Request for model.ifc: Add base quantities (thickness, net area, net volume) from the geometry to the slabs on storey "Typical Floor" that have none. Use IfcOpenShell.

First a look at what the model holds.

```python
import ifcopenshell
import ifcopenshell.util.element
import ifcopenshell.util.unit

model = ifcopenshell.open("model.ifc")
print(model.schema)
for unit_type in ("LENGTHUNIT", "AREAUNIT", "VOLUMEUNIT"):
    print(unit_type, ifcopenshell.util.unit.calculate_unit_scale(model, unit_type))
storey = next(s for s in model.by_type("IfcBuildingStorey") if s.Name == "Typical Floor")
slabs = [e for e in ifcopenshell.util.element.get_decomposition(storey) if e.is_a("IfcSlab")]
for e in sorted(slabs, key=lambda e: e.id()):
    print(e.id(), e.is_a(), e.Name, list(ifcopenshell.util.element.get_psets(e, qtos_only=True)), sep=" | ")
```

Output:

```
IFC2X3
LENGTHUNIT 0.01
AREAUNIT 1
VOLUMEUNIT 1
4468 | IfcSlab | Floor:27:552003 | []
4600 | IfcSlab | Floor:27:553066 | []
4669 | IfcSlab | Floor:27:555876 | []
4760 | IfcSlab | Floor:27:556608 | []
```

```python
import ifcopenshell
import ifcopenshell.api.pset
import ifcopenshell.geom
import ifcopenshell.util.element
import ifcopenshell.util.shape
import ifcopenshell.util.unit

model = ifcopenshell.open("model.ifc")
unit_scale = ifcopenshell.util.unit.calculate_unit_scale(model)
area_scale = ifcopenshell.util.unit.calculate_unit_scale(model, "AREAUNIT")
volume_scale = ifcopenshell.util.unit.calculate_unit_scale(model, "VOLUMEUNIT")
settings = ifcopenshell.geom.settings()

storey = next(s for s in model.by_type("IfcBuildingStorey") if s.Name == "Typical Floor")
slabs = [e for e in ifcopenshell.util.element.get_decomposition(storey) if e.is_a("IfcSlab")]

for e in sorted(slabs, key=lambda e: e.id()):
    if ifcopenshell.util.element.get_psets(e, qtos_only=True, should_inherit=False):
        continue
    # Geometry comes back in metres, in the element's own axes.
    shape = ifcopenshell.geom.create_shape(settings, e)
    values = {
        "Width": ifcopenshell.util.shape.get_z(shape.geometry) / unit_scale,
        "NetArea": ifcopenshell.util.shape.get_footprint_area(shape.geometry) / area_scale,
        "NetVolume": ifcopenshell.util.shape.get_volume(shape.geometry) / volume_scale,
    }
    qto = ifcopenshell.api.pset.add_qto(model, product=e, name="BaseQuantities")
    ifcopenshell.api.pset.edit_qto(model, qto=qto, properties=values)
    print(e.id(), {k: round(v, 3) for k, v in values.items()})

model.write("model_updated.ifc")
```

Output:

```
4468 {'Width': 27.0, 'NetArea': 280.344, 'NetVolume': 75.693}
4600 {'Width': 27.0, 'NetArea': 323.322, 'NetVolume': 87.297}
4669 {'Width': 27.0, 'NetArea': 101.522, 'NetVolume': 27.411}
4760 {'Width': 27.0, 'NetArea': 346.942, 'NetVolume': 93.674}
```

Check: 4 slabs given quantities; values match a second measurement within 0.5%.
